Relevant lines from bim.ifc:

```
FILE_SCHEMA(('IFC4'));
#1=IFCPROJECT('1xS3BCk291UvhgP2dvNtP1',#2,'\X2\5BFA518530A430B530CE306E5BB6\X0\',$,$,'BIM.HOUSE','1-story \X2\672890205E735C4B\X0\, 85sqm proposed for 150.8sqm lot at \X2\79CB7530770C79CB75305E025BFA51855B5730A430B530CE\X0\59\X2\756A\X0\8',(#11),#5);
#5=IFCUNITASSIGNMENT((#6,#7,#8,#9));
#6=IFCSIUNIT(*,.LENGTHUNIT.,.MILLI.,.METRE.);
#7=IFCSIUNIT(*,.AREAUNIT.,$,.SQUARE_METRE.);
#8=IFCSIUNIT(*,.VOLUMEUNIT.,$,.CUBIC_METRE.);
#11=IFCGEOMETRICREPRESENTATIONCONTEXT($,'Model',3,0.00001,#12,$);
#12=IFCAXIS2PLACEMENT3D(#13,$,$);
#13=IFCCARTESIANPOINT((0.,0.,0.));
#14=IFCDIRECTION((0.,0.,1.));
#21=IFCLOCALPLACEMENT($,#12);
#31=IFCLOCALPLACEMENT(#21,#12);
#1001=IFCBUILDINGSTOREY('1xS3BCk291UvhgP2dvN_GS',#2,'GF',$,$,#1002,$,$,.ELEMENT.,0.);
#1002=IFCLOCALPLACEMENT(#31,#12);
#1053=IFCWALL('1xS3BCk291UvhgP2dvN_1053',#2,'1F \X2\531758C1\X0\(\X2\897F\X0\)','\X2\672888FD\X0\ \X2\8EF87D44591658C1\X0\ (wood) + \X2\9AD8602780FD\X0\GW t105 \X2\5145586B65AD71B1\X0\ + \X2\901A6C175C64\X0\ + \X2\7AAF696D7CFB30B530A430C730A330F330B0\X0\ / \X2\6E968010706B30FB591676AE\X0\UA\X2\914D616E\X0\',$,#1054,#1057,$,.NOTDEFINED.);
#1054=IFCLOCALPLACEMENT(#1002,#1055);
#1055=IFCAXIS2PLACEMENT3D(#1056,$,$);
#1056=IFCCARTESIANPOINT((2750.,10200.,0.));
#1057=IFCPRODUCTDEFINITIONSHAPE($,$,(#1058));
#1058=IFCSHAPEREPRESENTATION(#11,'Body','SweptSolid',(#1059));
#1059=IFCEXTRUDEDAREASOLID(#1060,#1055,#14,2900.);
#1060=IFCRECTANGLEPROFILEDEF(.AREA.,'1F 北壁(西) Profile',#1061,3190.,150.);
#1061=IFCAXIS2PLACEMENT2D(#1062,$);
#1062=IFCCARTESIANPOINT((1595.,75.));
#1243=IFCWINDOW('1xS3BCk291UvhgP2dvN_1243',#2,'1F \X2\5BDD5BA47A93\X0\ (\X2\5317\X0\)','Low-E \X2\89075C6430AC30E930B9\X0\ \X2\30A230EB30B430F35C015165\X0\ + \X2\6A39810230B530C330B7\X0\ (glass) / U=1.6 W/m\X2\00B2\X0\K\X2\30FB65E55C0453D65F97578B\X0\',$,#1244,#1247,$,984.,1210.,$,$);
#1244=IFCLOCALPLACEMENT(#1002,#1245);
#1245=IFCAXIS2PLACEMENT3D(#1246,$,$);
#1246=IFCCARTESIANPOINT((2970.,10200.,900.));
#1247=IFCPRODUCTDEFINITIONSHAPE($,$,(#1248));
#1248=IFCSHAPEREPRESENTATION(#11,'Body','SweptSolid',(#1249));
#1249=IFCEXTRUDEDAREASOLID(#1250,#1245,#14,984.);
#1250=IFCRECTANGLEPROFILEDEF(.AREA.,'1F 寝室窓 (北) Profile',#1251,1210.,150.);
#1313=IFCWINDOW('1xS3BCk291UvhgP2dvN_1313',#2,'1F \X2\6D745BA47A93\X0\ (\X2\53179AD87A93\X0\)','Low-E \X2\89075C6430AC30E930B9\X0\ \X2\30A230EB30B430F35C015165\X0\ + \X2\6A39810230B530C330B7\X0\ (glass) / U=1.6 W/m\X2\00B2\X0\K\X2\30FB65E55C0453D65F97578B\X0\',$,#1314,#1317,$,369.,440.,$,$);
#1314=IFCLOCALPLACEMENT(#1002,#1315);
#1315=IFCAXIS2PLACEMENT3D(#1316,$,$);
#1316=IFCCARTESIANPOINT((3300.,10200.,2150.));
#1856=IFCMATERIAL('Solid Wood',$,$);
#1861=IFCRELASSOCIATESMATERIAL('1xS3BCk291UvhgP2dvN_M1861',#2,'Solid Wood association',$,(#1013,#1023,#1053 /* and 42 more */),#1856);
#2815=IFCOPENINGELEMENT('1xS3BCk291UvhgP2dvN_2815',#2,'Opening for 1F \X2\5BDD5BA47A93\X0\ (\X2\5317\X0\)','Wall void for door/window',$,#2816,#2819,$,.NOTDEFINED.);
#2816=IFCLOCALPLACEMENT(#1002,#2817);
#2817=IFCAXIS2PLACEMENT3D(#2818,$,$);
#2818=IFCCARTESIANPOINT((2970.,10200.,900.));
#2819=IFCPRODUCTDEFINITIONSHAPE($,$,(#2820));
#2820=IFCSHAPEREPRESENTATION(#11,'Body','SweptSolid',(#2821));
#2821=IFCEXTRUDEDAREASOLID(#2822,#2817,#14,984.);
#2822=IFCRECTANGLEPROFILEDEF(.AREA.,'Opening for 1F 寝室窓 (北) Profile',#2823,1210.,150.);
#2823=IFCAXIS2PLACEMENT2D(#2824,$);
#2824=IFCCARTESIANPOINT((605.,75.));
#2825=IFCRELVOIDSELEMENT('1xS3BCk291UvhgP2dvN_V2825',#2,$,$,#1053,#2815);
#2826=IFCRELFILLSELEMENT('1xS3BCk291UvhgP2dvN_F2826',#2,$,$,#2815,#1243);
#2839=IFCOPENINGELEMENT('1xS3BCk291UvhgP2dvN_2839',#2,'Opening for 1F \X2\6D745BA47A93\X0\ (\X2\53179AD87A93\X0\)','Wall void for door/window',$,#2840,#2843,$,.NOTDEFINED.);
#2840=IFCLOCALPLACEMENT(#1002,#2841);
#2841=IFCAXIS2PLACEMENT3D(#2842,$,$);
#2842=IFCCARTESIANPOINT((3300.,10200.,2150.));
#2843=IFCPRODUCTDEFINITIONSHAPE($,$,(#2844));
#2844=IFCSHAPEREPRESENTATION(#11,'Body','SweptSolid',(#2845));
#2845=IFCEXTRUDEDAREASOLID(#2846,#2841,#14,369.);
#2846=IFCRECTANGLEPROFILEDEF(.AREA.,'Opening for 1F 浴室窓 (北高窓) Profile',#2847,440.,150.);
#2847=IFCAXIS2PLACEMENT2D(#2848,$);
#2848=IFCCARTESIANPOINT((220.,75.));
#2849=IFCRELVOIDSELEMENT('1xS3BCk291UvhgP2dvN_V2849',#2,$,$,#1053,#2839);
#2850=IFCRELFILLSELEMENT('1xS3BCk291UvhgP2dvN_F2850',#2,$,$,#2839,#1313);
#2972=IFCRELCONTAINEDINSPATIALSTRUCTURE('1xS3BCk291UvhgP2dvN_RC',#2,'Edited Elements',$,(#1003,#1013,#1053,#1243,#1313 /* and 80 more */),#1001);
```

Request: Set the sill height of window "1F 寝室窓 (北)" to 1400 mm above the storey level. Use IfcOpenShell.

```python
import numpy as np
import ifcopenshell
import ifcopenshell.api.geometry
import ifcopenshell.geom
import ifcopenshell.util.element
import ifcopenshell.util.placement
import ifcopenshell.util.shape
import ifcopenshell.util.unit

model = ifcopenshell.open("bim.ifc")
unit_scale = ifcopenshell.util.unit.calculate_unit_scale(model)

window = model.by_guid("1xS3BCk291UvhgP2dvN_1243")
opening = window.FillsVoids[0].RelatingOpeningElement
storey = ifcopenshell.util.element.get_container(window, ifc_class="IfcBuildingStorey")
level = ifcopenshell.util.placement.get_local_placement(storey.ObjectPlacement)[2, 3]

# The opening's origin need not be at the sill, so measure its lowest point.
shape = ifcopenshell.geom.create_shape(ifcopenshell.geom.settings(), opening)
bottom = ifcopenshell.util.shape.get_shape_bottom_elevation(shape, shape.geometry) / unit_scale
dz = level + 1400.0 - bottom

shift = np.array([0.0, 0.0, dz])
# The window is not placed relative to its opening, so move both.
for product in (opening, window):
    matrix = ifcopenshell.util.placement.get_local_placement(product.ObjectPlacement)
    matrix[:3, 3] += shift
    ifcopenshell.api.geometry.edit_object_placement(model, product=product, matrix=matrix, is_si=False)

print(f"moved by {dz * unit_scale:+.3f} m")

model.write("bim_edited.ifc")
```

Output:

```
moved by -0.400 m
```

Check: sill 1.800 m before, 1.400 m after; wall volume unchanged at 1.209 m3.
